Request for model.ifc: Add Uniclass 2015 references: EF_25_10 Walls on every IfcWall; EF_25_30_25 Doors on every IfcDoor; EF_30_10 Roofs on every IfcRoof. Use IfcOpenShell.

First a look at what the model holds.

```python
import ifcopenshell

model = ifcopenshell.open("model.ifc")
print(model.schema)
print("classifications:", [c.Name for c in model.by_type("IfcClassification")])
for ifc_class in ("IfcDoor", "IfcRoof", "IfcStair", "IfcWall", "IfcWindow"):
    print(ifc_class, len(model.by_type(ifc_class)))
```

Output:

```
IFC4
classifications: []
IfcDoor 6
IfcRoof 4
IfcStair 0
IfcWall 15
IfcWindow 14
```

```python
import ifcopenshell
import ifcopenshell.api.classification

model = ifcopenshell.open("model.ifc")

system = ifcopenshell.api.classification.add_classification(model, classification="Uniclass 2015")

codes = {
    "IfcWall": ("EF_25_10", "Walls"),
    "IfcDoor": ("EF_25_30_25", "Doors"),
    "IfcRoof": ("EF_30_10", "Roofs"),
}
for ifc_class, (code, name) in codes.items():
    products = model.by_type(ifc_class)
    ifcopenshell.api.classification.add_reference(
        model, products=products, classification=system, identification=code, name=name
    )
    print(code, len(products))

model.write("model-out.ifc")
```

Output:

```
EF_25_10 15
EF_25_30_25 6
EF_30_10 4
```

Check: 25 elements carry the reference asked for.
